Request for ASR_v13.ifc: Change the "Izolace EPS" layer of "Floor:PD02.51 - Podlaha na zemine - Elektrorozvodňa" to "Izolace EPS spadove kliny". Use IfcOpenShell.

First a look at what the model holds.

```python
import ifcopenshell
import ifcopenshell.util.element

model = ifcopenshell.open("ASR_v13.ifc")
print(model.schema)
for layer_set in model.by_type("IfcMaterialLayerSet"):
    if layer_set.LayerSetName == "Floor:PD02.51 - Podlaha na zemine - Elektrorozvodňa":
        for layer in layer_set.MaterialLayers:
            print(layer.id(), layer.Material and layer.Material.Name, layer.LayerThickness, sep=" | ")
        print(len(ifcopenshell.util.element.get_elements_by_material(model, layer_set)), "elements and types use it")
print(sorted(m.Name for m in model.by_type("IfcMaterial") if m.Name)[:60])
```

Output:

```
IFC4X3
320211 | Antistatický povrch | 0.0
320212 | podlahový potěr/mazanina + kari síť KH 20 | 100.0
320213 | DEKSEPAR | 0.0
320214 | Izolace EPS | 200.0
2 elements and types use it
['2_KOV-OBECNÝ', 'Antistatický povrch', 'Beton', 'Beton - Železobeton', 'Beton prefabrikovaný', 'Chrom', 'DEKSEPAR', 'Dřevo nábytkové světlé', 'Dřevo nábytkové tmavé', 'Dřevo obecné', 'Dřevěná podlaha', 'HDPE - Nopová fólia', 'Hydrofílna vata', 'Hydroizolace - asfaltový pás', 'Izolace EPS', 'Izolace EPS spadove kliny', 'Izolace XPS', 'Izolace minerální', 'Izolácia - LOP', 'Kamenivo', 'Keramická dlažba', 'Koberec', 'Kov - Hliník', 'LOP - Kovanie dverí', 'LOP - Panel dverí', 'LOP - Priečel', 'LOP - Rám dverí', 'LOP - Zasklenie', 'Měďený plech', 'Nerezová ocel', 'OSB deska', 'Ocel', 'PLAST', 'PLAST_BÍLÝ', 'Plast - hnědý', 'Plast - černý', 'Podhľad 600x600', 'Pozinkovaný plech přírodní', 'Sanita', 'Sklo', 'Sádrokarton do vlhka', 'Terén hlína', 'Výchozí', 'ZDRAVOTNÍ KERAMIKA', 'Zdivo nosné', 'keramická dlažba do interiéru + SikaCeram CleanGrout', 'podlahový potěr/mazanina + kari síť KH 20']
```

```python
import ifcopenshell
import ifcopenshell.api.material

model = ifcopenshell.open("ASR_v13.ifc")

layer_set = next(s for s in model.by_type("IfcMaterialLayerSet") if s.LayerSetName == "Floor:PD02.51 - Podlaha na zemine - Elektrorozvodňa")
layer = next(l for l in layer_set.MaterialLayers if l.Material and l.Material.Name == "Izolace EPS")
material = next(m for m in model.by_type("IfcMaterial") if m.Name == "Izolace EPS spadove kliny")

# Point this one layer at the other material; renaming the old one would change it everywhere.
ifcopenshell.api.material.edit_layer(model, layer=layer, attributes={"Name": material.Name}, material=material)

print([l.Material.Name if l.Material else None for l in layer_set.MaterialLayers])

model.write("ASR_v13_rev.ifc")
```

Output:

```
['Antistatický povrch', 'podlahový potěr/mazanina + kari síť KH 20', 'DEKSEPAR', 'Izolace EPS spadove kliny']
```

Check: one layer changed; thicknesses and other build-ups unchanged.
